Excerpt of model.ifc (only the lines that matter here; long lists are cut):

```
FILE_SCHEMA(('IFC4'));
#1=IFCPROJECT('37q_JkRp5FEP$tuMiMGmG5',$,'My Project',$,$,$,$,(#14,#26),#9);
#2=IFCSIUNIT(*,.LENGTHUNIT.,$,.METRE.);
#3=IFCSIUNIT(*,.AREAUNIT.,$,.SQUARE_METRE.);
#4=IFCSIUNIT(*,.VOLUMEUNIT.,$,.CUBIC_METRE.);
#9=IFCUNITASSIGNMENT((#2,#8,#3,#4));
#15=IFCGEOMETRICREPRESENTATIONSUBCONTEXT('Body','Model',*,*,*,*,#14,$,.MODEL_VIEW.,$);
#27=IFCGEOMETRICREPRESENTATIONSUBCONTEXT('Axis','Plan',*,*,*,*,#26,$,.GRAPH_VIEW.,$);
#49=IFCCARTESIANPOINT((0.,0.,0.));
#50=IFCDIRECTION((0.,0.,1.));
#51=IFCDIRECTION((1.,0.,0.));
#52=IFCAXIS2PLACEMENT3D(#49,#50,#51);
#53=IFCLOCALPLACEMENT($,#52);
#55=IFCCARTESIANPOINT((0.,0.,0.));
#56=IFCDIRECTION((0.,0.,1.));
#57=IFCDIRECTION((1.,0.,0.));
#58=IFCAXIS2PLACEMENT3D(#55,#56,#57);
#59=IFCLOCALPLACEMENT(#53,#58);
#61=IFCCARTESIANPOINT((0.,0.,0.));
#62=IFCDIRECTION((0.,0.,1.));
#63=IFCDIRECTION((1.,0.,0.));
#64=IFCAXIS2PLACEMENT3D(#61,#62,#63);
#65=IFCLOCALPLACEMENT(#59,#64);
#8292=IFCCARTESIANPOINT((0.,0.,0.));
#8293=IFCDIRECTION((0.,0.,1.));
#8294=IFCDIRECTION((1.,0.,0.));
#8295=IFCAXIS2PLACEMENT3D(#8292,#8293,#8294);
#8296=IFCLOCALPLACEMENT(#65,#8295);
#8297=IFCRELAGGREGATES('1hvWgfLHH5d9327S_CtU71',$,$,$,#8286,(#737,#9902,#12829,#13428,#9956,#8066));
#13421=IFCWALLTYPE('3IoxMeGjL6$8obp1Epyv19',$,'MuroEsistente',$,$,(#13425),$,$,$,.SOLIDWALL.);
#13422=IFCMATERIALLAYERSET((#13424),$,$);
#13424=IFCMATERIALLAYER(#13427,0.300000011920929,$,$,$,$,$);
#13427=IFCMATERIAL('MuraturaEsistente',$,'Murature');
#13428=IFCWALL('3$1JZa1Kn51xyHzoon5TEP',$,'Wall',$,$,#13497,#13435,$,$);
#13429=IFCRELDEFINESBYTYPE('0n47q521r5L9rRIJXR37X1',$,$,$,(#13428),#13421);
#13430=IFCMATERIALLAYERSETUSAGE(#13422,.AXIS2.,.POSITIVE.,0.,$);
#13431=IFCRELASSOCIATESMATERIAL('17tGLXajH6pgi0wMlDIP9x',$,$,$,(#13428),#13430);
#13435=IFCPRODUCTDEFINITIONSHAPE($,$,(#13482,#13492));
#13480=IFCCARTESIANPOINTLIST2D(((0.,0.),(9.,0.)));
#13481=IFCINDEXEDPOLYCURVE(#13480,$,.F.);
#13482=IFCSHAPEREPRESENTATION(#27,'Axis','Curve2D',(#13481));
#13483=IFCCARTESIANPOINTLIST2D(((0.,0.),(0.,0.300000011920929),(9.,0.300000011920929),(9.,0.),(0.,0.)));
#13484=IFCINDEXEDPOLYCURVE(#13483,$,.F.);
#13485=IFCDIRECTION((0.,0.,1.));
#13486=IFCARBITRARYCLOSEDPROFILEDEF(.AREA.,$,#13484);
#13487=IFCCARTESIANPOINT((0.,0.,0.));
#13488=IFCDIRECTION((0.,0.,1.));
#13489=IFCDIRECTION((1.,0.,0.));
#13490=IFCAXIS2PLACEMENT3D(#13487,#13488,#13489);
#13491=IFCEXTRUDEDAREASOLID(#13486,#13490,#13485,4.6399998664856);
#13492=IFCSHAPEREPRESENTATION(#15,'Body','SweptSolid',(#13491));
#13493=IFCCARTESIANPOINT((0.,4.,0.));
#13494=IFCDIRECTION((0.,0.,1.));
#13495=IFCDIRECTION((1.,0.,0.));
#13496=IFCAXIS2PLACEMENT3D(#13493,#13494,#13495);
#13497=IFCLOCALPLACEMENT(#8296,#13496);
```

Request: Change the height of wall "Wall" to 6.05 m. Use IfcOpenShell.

```python
import ifcopenshell
import ifcopenshell.geom
import ifcopenshell.util.representation
import ifcopenshell.util.shape
import ifcopenshell.util.unit

model = ifcopenshell.open("model.ifc")
unit_scale = ifcopenshell.util.unit.calculate_unit_scale(model)
settings = ifcopenshell.geom.settings()


def volume(element):
    """Net volume in cubic metres, openings subtracted."""
    shape = ifcopenshell.geom.create_shape(settings, element)
    return ifcopenshell.util.shape.get_volume(shape.geometry)


wall = model.by_guid("3$1JZa1Kn51xyHzoon5TEP")
before = volume(wall)

body = ifcopenshell.util.representation.get_representation(wall, "Model", "Body")
solid = body.Items[0]
old_height = solid.Depth
solid.Depth = 6.05 / unit_scale
after = volume(wall)

print(f"height {old_height:g} -> {solid.Depth:g}, volume {before:.3f} -> {after:.3f} m3")

model.write("model_updated.ifc")
```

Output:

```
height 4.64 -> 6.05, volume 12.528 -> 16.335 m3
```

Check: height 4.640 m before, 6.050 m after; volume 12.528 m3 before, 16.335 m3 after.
